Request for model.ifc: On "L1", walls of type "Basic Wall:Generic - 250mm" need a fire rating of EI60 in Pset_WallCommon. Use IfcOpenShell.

First a look at what the model holds.

```python
import ifcopenshell
import ifcopenshell.util.element

model = ifcopenshell.open("model.ifc")
print(model.schema)
storey = next(s for s in model.by_type("IfcBuildingStorey") if s.Name == "L1")
walls = [e for e in ifcopenshell.util.element.get_decomposition(storey) if e.is_a("IfcWall")]
seen = {}
for e in walls:
    element_type = ifcopenshell.util.element.get_type(e)
    key = (element_type.Name if element_type != e and element_type else None, ifcopenshell.util.element.get_pset(e, "Pset_WallCommon", "FireRating"))
    seen[key] = seen.get(key, 0) + 1
for (name, value), count in sorted(seen.items(), key=str):
    print(count, "x", name, "|", value)
```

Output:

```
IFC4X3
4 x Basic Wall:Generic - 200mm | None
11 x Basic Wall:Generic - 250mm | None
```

```python
import ifcopenshell
import ifcopenshell.api.pset
import ifcopenshell.util.element

model = ifcopenshell.open("model.ifc")

storey = next(s for s in model.by_type("IfcBuildingStorey") if s.Name == "L1")
walls = [e for e in ifcopenshell.util.element.get_decomposition(storey) if e.is_a("IfcWall")]

count = 0
for e in walls:
    element_type = ifcopenshell.util.element.get_type(e)
    if element_type in (None, e) or element_type.Name != "Basic Wall:Generic - 250mm":
        continue
    # add_pset returns the element's existing set when there is one.
    pset = ifcopenshell.api.pset.add_pset(model, product=e, name="Pset_WallCommon")
    ifcopenshell.api.pset.edit_pset(model, pset=pset, properties={"FireRating": "EI60"})
    count += 1

print(count, "walls updated")

model.write("model-out.ifc")
```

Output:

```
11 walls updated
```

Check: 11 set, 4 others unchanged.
